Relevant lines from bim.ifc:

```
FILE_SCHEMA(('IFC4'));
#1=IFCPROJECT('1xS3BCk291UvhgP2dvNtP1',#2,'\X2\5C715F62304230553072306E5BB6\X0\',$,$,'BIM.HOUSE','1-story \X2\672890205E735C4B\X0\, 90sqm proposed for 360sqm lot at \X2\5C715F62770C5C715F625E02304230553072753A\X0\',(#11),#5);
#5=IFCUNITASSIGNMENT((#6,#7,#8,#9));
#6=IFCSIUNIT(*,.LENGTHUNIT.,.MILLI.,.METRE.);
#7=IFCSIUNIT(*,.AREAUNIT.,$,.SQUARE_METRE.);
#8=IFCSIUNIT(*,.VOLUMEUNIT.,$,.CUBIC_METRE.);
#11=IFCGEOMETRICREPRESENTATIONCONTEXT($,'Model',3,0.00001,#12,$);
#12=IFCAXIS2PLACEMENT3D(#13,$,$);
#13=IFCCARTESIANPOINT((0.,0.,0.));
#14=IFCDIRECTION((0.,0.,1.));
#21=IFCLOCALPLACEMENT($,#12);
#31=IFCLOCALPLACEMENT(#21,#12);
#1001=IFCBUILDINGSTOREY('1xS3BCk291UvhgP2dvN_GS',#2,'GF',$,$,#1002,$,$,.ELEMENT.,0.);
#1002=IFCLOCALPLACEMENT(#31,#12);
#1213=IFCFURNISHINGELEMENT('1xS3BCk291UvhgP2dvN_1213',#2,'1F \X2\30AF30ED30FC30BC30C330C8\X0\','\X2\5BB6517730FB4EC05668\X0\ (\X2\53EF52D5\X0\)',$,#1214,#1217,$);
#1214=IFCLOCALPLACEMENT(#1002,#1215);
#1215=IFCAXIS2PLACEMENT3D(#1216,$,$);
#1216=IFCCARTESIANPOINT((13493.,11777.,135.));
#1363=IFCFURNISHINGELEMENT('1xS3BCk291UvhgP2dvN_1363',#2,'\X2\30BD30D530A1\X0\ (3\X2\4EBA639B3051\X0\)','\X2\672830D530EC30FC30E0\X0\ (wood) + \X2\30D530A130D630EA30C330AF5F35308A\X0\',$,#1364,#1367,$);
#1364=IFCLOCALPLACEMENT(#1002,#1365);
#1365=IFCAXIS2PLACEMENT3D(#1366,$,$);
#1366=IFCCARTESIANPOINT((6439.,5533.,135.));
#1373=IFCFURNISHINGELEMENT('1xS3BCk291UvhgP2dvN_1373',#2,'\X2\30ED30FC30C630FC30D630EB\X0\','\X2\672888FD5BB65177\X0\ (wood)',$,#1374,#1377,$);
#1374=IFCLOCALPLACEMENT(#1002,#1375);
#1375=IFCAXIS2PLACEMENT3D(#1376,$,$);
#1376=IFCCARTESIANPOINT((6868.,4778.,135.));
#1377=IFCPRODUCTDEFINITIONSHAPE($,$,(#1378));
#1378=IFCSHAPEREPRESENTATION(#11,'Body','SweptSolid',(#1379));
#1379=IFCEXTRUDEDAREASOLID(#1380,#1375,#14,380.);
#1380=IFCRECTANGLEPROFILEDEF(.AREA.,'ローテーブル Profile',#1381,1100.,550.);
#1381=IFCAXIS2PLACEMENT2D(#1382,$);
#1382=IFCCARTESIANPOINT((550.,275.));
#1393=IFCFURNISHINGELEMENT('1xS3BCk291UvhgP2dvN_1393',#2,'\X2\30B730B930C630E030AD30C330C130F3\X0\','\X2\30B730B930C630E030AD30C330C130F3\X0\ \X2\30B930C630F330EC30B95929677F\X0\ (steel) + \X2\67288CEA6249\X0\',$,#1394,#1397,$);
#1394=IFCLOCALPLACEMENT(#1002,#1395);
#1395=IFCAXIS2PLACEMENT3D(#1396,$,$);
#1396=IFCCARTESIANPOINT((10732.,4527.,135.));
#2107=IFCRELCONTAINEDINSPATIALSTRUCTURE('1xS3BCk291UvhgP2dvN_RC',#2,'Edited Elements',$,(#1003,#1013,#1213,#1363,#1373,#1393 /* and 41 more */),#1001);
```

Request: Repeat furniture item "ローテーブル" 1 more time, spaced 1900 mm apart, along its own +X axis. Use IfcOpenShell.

```python
import ifcopenshell
import ifcopenshell.api.geometry
import ifcopenshell.api.root
import ifcopenshell.util.element
import ifcopenshell.util.placement
import ifcopenshell.util.unit

model = ifcopenshell.open("bim.ifc")
unit_scale = ifcopenshell.util.unit.calculate_unit_scale(model)


def reuse_history(source, copy):
    """copy_class also copies each property set's owner history, people and application; keep the originals."""
    for rel in copy.IsDefinedBy:
        if rel.is_a("IfcRelDefinesByProperties") and (history := rel.RelatingPropertyDefinition.OwnerHistory):
            rel.RelatingPropertyDefinition.OwnerHistory = source.OwnerHistory
            ifcopenshell.util.element.remove_deep2(model, history)


source = model.by_guid("1xS3BCk291UvhgP2dvN_1373")
base = ifcopenshell.util.placement.get_local_placement(source.ObjectPlacement)
step = base[:3, 0] * 1.9 / unit_scale

for i in range(1, 2):
    copy = ifcopenshell.api.root.copy_class(model, product=source)
    copy.Representation = ifcopenshell.util.element.copy_deep(
        model, source.Representation, exclude=["IfcGeometricRepresentationContext", "IfcRepresentationMap"]
    )
    reuse_history(source, copy)
    matrix = base.copy()
    matrix[:3, 3] += i * step
    print("added at", matrix[:3, 3].round(3) + 0.0)
    ifcopenshell.api.geometry.edit_object_placement(model, product=copy, matrix=matrix, is_si=False)

model.write("bim_rev.ifc")
```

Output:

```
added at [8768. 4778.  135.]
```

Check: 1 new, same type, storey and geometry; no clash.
